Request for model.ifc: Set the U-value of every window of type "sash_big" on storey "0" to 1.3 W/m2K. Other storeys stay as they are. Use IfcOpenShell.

First a look at what the model holds.

```python
import ifcopenshell
import ifcopenshell.util.element

model = ifcopenshell.open("model.ifc")
print(model.schema)
storey = next(s for s in model.by_type("IfcBuildingStorey") if s.Name == "0")
windows = [e for e in ifcopenshell.util.element.get_decomposition(storey) if e.is_a("IfcWindow")]
seen = {}
for e in windows:
    element_type = ifcopenshell.util.element.get_type(e)
    key = (element_type.Name if element_type != e and element_type else None, ifcopenshell.util.element.get_pset(e, "Pset_WindowCommon", "ThermalTransmittance"))
    seen[key] = seen.get(key, 0) + 1
for (name, value), count in sorted(seen.items(), key=str):
    print(count, "x", name, "|", value)
```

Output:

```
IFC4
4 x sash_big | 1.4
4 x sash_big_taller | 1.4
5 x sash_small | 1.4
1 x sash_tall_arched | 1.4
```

```python
import ifcopenshell
import ifcopenshell.api.pset
import ifcopenshell.util.element

model = ifcopenshell.open("model.ifc")

storey = next(s for s in model.by_type("IfcBuildingStorey") if s.Name == "0")
windows = [e for e in ifcopenshell.util.element.get_decomposition(storey) if e.is_a("IfcWindow")]

count = 0
for e in windows:
    element_type = ifcopenshell.util.element.get_type(e)
    if element_type in (None, e) or element_type.Name != "sash_big":
        continue
    # add_pset returns the element's existing set when there is one.
    pset = ifcopenshell.api.pset.add_pset(model, product=e, name="Pset_WindowCommon")
    ifcopenshell.api.pset.edit_pset(model, pset=pset, properties={"ThermalTransmittance": 1.3})
    count += 1

print(count, "windows updated")

model.write("model_v2.ifc")
```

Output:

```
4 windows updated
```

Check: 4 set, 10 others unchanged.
